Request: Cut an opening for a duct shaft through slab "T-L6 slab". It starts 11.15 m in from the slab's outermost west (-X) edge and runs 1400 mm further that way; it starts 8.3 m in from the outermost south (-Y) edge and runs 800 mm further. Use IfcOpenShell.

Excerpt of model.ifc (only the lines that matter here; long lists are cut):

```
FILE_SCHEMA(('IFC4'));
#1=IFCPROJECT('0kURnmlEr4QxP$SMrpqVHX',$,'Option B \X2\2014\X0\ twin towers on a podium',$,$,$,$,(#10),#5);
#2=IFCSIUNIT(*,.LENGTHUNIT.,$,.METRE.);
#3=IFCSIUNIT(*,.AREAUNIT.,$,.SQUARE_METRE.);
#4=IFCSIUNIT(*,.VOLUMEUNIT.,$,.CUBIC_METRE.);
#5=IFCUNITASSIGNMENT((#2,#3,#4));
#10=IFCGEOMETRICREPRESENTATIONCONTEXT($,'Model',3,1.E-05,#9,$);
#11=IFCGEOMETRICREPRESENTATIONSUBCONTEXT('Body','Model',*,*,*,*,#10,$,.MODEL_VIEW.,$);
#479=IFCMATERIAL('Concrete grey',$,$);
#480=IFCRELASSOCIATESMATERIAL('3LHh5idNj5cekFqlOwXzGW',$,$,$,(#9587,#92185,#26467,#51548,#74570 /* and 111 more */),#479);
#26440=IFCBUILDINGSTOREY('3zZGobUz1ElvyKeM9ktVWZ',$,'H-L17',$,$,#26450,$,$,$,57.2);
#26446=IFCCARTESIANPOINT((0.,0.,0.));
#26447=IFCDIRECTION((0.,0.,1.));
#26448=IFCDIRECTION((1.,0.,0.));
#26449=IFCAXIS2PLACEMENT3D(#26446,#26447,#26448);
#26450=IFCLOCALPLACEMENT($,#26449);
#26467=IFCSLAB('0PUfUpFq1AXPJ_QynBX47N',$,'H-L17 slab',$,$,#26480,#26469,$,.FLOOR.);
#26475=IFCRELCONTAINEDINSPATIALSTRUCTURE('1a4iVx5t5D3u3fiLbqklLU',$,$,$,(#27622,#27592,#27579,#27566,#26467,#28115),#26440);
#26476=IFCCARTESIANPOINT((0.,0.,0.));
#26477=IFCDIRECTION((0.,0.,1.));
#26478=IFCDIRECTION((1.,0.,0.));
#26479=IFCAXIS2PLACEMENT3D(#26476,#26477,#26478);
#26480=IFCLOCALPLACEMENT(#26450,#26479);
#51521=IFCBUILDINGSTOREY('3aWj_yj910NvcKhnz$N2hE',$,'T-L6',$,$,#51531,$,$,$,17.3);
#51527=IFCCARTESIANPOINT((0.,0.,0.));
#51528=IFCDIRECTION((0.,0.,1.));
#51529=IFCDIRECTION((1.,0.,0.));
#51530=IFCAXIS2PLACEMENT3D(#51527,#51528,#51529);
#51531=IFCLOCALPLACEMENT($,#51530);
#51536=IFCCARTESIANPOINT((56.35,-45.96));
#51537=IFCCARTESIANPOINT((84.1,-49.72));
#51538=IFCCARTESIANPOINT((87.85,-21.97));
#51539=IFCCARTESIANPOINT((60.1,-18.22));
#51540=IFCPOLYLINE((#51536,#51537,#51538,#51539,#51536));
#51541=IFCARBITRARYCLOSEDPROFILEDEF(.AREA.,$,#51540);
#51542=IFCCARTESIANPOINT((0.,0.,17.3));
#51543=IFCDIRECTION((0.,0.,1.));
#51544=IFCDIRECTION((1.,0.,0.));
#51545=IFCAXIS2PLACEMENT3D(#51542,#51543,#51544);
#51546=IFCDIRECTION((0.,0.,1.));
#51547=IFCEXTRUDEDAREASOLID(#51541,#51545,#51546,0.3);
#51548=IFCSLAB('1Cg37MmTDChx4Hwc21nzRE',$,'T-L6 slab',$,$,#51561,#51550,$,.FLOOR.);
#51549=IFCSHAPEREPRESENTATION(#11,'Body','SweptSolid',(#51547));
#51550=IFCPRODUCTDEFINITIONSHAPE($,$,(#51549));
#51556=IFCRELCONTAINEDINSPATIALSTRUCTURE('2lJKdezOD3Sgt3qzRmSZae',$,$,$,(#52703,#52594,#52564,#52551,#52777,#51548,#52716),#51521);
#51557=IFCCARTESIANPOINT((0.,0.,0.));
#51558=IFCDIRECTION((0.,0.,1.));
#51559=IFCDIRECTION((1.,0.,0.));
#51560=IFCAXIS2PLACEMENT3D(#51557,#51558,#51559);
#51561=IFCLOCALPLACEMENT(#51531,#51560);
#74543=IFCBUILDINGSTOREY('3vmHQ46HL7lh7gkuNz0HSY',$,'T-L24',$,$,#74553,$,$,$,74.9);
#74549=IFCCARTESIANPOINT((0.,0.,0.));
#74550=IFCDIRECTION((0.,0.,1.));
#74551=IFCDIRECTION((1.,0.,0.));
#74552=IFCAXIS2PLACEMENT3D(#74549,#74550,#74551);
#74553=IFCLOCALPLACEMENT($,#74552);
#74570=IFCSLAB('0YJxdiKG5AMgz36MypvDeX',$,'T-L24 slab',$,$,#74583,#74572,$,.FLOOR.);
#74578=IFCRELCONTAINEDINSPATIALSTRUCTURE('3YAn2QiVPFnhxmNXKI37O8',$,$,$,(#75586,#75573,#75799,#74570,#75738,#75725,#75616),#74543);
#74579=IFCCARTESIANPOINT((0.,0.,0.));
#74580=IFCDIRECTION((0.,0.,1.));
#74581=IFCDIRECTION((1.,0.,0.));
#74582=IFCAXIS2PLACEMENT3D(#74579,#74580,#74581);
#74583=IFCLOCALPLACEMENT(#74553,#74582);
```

```python
import numpy as np
import ifcopenshell
import ifcopenshell.api.feature
import ifcopenshell.api.geometry
import ifcopenshell.api.root
import ifcopenshell.geom
import ifcopenshell.util.placement
import ifcopenshell.util.representation
import ifcopenshell.util.shape
import ifcopenshell.util.unit

model = ifcopenshell.open("model.ifc")
unit_scale = ifcopenshell.util.unit.calculate_unit_scale(model)
settings = ifcopenshell.geom.settings()


def volume(element):
    """Net volume in cubic metres, openings subtracted."""
    shape = ifcopenshell.geom.create_shape(settings, element)
    return ifcopenshell.util.shape.get_volume(shape.geometry)


slab = model.by_id(51548)
before = volume(slab)

# Extent in the slab's own axes, in metres. The edges named are its -X and -Y sides.
slab_shape = ifcopenshell.geom.create_shape(settings, slab)
vertices = ifcopenshell.util.shape.get_vertices(slab_shape.geometry)
x_min, y_min, bottom = vertices.min(axis=0)
top = vertices[:, 2].max()

opening = ifcopenshell.api.root.create_entity(model, ifc_class="IfcOpeningElement", name="Duct shaft opening", predefined_type="OPENING")
context = ifcopenshell.util.representation.get_context(model, "Model", "Body", "MODEL_VIEW")
width, depth = 1.4, 0.8
outline = [(0.0, 0.0), (width, 0.0), (width, depth), (0.0, depth), (0.0, 0.0)]
# Overshoot both faces by 50 mm so the cut is clean.
shape = ifcopenshell.api.geometry.add_slab_representation(
    model, context=context, depth=top - bottom + 0.1, polyline=outline
)
ifcopenshell.api.geometry.assign_representation(model, product=opening, representation=shape)

matrix = ifcopenshell.util.placement.get_local_placement(slab.ObjectPlacement)
matrix[:, 3] = matrix @ np.append(np.array([x_min + 11.15, y_min + 8.3, bottom - 0.05]) / unit_scale, 1.0)
ifcopenshell.api.geometry.edit_object_placement(model, product=opening, matrix=matrix, is_si=False)
ifcopenshell.api.feature.add_feature(model, feature=opening, element=slab)

after = volume(slab)

print(f"slab volume {before:.3f} -> {after:.3f} m3")

model.write("model_rev.ifc")
```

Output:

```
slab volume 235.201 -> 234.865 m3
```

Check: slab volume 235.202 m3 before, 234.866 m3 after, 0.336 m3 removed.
